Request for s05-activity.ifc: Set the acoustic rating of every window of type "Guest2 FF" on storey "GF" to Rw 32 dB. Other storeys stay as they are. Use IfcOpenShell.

First a look at what the model holds.

```python
import ifcopenshell
import ifcopenshell.util.element

model = ifcopenshell.open("s05-activity.ifc")
print(model.schema)
storey = next(s for s in model.by_type("IfcBuildingStorey") if s.Name == "GF")
windows = [e for e in ifcopenshell.util.element.get_decomposition(storey) if e.is_a("IfcWindow")]
seen = {}
for e in windows:
    element_type = ifcopenshell.util.element.get_type(e)
    key = (element_type.Name if element_type != e and element_type else None, ifcopenshell.util.element.get_pset(e, "Pset_WindowCommon", "AcousticRating"))
    seen[key] = seen.get(key, 0) + 1
for (name, value), count in sorted(seen.items(), key=str):
    print(count, "x", name, "|", value)
```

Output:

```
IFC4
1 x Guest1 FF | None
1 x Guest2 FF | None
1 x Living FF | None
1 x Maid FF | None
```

```python
import ifcopenshell
import ifcopenshell.api.pset
import ifcopenshell.util.element

model = ifcopenshell.open("s05-activity.ifc")

storey = next(s for s in model.by_type("IfcBuildingStorey") if s.Name == "GF")
windows = [e for e in ifcopenshell.util.element.get_decomposition(storey) if e.is_a("IfcWindow")]

count = 0
for e in windows:
    element_type = ifcopenshell.util.element.get_type(e)
    if element_type in (None, e) or element_type.Name != "Guest2 FF":
        continue
    # add_pset returns the element's existing set when there is one.
    pset = ifcopenshell.api.pset.add_pset(model, product=e, name="Pset_WindowCommon")
    ifcopenshell.api.pset.edit_pset(model, pset=pset, properties={"AcousticRating": "Rw 32 dB"})
    count += 1

print(count, "windows updated")

model.write("s05-activity_rev.ifc")
```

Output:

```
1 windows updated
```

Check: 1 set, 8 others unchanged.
